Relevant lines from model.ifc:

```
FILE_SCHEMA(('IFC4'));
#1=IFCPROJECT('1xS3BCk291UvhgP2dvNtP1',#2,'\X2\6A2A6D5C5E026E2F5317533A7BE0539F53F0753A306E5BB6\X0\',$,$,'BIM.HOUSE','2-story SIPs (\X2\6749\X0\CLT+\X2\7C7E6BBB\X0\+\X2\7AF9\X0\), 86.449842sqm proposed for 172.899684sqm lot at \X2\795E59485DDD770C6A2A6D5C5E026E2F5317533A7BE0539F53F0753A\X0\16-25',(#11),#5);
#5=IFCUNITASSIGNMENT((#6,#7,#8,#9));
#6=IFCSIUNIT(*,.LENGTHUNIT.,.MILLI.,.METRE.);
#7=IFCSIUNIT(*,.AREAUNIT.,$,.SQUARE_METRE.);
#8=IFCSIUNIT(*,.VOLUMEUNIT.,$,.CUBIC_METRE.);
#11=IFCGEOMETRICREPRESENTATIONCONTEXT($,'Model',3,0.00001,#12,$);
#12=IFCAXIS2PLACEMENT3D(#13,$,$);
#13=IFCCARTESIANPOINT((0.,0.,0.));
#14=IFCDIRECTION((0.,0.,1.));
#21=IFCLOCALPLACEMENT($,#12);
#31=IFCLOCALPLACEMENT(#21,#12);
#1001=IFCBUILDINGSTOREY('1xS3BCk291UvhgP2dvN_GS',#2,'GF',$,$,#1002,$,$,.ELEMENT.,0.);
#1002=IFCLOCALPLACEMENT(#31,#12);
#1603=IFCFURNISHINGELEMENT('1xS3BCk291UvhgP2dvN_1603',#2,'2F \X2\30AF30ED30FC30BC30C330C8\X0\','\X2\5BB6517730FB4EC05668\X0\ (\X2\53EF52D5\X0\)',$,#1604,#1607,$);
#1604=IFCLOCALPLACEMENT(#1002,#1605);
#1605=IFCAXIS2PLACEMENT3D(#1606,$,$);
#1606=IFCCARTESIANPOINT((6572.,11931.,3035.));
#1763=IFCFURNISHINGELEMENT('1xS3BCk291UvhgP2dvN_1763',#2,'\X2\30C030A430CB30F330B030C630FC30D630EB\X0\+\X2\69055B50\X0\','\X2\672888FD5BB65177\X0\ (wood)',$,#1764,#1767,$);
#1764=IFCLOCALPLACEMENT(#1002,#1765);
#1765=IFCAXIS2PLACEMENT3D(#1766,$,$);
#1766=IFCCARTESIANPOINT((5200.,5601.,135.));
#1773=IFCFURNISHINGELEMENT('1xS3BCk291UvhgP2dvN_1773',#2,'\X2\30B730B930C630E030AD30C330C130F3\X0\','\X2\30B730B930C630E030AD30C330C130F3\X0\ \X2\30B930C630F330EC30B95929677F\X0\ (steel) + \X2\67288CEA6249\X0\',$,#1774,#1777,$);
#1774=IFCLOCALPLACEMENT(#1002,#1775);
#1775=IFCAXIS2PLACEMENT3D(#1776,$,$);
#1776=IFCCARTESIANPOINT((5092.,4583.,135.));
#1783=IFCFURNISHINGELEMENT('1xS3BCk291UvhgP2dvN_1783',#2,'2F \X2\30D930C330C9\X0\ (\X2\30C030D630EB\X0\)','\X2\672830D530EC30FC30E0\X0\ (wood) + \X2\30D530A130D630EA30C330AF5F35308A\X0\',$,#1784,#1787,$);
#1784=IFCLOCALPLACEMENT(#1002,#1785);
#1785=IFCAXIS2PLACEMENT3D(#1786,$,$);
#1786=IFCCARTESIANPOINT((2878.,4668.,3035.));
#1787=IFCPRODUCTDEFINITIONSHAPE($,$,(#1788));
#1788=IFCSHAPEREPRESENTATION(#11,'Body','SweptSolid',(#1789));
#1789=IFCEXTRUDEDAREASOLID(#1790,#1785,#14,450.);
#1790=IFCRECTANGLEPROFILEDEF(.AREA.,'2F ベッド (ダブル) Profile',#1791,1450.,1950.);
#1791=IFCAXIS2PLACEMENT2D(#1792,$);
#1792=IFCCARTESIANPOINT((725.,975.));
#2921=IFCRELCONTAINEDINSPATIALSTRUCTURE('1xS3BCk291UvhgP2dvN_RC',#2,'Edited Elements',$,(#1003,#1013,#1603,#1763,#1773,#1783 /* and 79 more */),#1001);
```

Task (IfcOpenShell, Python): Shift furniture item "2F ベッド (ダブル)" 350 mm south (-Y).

```python
import ifcopenshell
import ifcopenshell.api.geometry
import ifcopenshell.util.placement

model = ifcopenshell.open("model.ifc")

item = model.by_guid("1xS3BCk291UvhgP2dvN_1783")
matrix = ifcopenshell.util.placement.get_local_placement(item.ObjectPlacement)
matrix[1, 3] -= 350.0
ifcopenshell.api.geometry.edit_object_placement(model, product=item, matrix=matrix, is_si=False)

print(ifcopenshell.util.placement.get_local_placement(item.ObjectPlacement).round(3) + 0.0)

model.write("model-out.ifc")
```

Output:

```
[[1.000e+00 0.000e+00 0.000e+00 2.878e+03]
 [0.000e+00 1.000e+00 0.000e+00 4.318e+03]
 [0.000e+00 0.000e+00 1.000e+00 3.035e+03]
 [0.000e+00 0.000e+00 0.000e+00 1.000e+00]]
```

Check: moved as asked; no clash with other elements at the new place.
